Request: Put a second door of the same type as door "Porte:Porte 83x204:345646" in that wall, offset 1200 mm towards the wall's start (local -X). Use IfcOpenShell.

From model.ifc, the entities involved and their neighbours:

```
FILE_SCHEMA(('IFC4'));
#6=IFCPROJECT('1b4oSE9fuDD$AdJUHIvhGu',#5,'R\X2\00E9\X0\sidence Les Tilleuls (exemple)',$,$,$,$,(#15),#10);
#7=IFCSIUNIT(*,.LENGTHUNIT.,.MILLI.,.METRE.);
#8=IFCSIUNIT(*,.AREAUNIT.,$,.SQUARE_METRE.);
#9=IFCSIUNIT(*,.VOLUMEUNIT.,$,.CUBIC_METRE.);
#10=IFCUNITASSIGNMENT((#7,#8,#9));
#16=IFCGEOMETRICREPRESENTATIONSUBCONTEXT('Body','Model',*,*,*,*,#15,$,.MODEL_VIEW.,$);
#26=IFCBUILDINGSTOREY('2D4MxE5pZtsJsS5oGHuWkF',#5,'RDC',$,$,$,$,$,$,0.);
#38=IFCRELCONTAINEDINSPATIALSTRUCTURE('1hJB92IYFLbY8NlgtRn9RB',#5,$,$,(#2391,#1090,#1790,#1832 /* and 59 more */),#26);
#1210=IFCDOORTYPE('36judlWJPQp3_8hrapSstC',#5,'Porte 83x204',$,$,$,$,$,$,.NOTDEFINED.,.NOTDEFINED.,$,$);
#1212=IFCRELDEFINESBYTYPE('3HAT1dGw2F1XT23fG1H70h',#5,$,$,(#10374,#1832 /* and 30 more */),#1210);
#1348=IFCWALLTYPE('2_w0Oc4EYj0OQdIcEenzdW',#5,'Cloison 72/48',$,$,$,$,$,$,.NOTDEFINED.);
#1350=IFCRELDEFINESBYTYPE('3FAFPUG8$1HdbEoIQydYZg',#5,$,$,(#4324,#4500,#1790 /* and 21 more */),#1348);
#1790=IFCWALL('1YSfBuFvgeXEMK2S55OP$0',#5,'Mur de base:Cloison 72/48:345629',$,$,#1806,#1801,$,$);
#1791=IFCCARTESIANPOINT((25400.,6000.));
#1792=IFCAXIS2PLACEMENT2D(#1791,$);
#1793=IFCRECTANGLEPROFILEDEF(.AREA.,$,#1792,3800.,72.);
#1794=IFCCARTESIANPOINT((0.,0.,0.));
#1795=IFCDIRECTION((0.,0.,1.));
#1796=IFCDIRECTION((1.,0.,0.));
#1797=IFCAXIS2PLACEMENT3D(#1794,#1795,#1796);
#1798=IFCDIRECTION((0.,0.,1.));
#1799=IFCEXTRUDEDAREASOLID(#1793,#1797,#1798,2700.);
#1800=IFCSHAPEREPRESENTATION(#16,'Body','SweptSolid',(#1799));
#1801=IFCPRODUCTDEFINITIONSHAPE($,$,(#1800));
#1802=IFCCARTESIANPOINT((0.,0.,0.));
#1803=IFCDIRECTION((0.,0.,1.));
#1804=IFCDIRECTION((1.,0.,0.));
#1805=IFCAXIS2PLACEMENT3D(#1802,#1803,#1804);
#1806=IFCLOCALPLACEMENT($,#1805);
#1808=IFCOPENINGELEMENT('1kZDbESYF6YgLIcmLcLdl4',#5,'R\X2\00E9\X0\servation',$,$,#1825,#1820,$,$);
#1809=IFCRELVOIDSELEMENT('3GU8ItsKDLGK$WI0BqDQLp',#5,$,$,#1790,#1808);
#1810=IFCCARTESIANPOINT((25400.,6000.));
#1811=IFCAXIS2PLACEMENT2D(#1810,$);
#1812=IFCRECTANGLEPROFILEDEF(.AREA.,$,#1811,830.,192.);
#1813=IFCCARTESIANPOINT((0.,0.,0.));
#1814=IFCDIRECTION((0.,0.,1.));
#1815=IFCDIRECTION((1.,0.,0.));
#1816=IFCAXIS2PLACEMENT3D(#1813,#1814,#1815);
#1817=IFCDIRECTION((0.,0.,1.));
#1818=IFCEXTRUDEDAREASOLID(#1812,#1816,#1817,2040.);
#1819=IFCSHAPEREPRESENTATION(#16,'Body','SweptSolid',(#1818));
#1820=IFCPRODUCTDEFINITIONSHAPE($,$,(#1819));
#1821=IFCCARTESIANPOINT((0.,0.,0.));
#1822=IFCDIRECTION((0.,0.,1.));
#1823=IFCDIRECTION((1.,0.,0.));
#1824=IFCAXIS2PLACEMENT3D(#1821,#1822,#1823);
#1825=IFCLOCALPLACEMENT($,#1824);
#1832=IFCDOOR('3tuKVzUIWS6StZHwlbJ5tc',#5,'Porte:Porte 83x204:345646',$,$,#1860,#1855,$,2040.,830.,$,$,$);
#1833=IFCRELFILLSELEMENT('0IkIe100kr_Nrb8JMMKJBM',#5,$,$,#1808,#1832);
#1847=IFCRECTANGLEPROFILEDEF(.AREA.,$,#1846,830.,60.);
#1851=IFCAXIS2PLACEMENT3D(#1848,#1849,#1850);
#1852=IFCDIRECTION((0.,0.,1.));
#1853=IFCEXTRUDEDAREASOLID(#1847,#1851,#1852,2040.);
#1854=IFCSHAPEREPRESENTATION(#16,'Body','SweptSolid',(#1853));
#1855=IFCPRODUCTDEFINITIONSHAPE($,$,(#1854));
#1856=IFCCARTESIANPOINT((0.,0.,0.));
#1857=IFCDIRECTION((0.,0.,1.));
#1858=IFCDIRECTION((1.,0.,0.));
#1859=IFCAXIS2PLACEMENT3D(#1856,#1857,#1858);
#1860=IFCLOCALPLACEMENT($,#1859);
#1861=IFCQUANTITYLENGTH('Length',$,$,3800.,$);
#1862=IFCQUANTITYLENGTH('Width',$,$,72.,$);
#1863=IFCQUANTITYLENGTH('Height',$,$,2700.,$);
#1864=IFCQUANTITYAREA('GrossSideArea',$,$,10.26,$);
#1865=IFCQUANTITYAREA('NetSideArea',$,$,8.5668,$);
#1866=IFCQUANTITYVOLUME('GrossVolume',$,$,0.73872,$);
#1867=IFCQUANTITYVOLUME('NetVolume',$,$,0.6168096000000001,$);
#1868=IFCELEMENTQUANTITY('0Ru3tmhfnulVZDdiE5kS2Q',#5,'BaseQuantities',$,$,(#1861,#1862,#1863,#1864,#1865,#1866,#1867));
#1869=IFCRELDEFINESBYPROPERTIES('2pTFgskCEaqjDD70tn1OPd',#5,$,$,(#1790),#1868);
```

```python
import ifcopenshell
import ifcopenshell.api.feature
import ifcopenshell.api.geometry
import ifcopenshell.api.pset
import ifcopenshell.api.root
import ifcopenshell.geom
import ifcopenshell.util.element
import ifcopenshell.util.placement
import ifcopenshell.util.shape
import ifcopenshell.util.unit

model = ifcopenshell.open("model.ifc")
unit_scale = ifcopenshell.util.unit.calculate_unit_scale(model)
area_scale = ifcopenshell.util.unit.calculate_unit_scale(model, "AREAUNIT")
volume_scale = ifcopenshell.util.unit.calculate_unit_scale(model, "VOLUMEUNIT")
settings = ifcopenshell.geom.settings()


def volume(element):
    """Net volume in cubic metres, openings subtracted."""
    shape = ifcopenshell.geom.create_shape(settings, element)
    return ifcopenshell.util.shape.get_volume(shape.geometry)


def reuse_history(source, copy):
    """copy_class also copies each property set's owner history, people and application; keep the originals."""
    for rel in copy.IsDefinedBy:
        if rel.is_a("IfcRelDefinesByProperties") and (history := rel.RelatingPropertyDefinition.OwnerHistory):
            rel.RelatingPropertyDefinition.OwnerHistory = source.OwnerHistory
            ifcopenshell.util.element.remove_deep2(model, history)


door = model.by_guid("3tuKVzUIWS6StZHwlbJ5tc")
opening = door.FillsVoids[0].RelatingOpeningElement
wall = opening.VoidsElements[0].RelatingBuildingElement
before = volume(wall)
shift = ifcopenshell.util.placement.get_local_placement(wall.ObjectPlacement)[:3, 0] * -1.2 / unit_scale

# copy_class copies the void relationship, type, container and properties, but no geometry.
new_opening = ifcopenshell.api.root.copy_class(model, product=opening)
new_opening.Representation = ifcopenshell.util.element.copy_deep(
    model, opening.Representation, exclude=["IfcGeometricRepresentationContext", "IfcRepresentationMap"]
)
reuse_history(opening, new_opening)
new_door = ifcopenshell.api.root.copy_class(model, product=door)
new_door.Representation = ifcopenshell.util.element.copy_deep(
    model, door.Representation, exclude=["IfcGeometricRepresentationContext", "IfcRepresentationMap"]
)
new_door.Name = "Porte:Porte 83x204"
reuse_history(door, new_door)
ifcopenshell.api.feature.add_filling(model, opening=new_opening, element=new_door)

for old, new in ((opening, new_opening), (door, new_door)):
    matrix = ifcopenshell.util.placement.get_local_placement(old.ObjectPlacement)
    matrix[:3, 3] += shift
    ifcopenshell.api.geometry.edit_object_placement(model, product=new, matrix=matrix, is_si=False)

after = volume(wall)
thickness = 0.072  # wall thickness in metres

# Update the wall's stored quantities.
qto = model.by_id(ifcopenshell.util.element.get_pset(wall, "BaseQuantities", should_inherit=False)["id"])
ifcopenshell.api.pset.edit_qto(model, qto=qto, properties={
    "NetSideArea": after / thickness / area_scale,
    "NetVolume": after / volume_scale,
})

print(f"wall volume {before:.3f} -> {after:.3f} m3")

model.write("model_rev.ifc")
```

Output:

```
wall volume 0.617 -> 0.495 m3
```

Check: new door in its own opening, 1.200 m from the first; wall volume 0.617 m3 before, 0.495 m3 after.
